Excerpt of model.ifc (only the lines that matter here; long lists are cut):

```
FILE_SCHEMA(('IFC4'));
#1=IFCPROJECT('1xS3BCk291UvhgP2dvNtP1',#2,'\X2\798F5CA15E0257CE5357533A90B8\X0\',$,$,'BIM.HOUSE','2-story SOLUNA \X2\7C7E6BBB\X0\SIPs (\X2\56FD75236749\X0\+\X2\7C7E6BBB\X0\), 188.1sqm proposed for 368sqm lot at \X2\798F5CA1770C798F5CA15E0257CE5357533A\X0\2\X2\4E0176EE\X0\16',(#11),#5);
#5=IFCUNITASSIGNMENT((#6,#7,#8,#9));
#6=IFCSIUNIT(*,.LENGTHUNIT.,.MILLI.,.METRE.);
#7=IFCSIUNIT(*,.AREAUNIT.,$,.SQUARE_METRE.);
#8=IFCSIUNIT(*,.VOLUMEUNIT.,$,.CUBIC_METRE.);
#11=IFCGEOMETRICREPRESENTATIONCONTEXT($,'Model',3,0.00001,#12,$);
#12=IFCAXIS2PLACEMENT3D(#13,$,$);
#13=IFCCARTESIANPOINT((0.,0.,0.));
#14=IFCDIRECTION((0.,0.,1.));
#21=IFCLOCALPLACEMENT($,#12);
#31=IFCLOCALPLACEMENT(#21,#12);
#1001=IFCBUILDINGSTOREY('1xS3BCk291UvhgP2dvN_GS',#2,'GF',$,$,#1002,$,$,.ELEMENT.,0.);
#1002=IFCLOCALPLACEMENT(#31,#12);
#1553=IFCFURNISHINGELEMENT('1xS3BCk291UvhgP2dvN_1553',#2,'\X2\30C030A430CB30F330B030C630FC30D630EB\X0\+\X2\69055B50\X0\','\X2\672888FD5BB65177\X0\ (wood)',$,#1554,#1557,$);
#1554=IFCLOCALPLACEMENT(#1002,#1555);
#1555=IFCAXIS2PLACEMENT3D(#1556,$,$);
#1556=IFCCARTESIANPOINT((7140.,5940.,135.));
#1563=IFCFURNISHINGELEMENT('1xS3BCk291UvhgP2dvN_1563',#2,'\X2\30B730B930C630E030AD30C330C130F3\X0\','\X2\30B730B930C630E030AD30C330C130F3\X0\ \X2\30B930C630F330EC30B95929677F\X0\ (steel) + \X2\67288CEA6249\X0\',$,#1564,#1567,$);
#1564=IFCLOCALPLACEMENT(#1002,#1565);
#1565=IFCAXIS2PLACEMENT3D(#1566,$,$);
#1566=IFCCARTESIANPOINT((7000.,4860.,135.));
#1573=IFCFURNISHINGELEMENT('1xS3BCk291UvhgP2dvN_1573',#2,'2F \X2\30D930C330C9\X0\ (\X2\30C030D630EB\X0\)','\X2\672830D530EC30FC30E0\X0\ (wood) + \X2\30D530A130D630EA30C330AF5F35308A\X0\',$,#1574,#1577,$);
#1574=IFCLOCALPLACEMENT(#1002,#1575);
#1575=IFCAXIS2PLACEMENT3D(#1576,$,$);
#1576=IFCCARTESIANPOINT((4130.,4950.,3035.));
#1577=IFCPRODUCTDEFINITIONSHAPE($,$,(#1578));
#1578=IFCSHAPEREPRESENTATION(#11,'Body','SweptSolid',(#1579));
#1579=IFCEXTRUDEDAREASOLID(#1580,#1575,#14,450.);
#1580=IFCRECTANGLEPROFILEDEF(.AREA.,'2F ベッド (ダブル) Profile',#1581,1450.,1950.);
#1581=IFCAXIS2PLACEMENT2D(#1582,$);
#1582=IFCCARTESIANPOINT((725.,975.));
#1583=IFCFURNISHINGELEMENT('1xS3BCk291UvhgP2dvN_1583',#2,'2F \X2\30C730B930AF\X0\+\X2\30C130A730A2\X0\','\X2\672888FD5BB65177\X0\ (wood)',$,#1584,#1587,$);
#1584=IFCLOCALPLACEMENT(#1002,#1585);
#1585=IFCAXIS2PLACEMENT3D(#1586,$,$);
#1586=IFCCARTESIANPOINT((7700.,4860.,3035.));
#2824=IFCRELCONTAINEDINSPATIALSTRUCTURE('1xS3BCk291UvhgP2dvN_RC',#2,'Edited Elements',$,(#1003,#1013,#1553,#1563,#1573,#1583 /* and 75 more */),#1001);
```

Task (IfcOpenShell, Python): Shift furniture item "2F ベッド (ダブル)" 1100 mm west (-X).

```python
import ifcopenshell
import ifcopenshell.api.geometry
import ifcopenshell.util.placement

model = ifcopenshell.open("model.ifc")

item = model.by_guid("1xS3BCk291UvhgP2dvN_1573")
matrix = ifcopenshell.util.placement.get_local_placement(item.ObjectPlacement)
matrix[0, 3] -= 1100.0
ifcopenshell.api.geometry.edit_object_placement(model, product=item, matrix=matrix, is_si=False)

print(ifcopenshell.util.placement.get_local_placement(item.ObjectPlacement).round(3) + 0.0)

model.write("model-out.ifc")
```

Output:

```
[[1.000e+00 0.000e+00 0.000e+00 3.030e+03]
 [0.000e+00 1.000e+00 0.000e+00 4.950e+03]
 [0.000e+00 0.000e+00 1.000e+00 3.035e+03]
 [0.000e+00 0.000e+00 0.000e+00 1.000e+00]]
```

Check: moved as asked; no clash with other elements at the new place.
